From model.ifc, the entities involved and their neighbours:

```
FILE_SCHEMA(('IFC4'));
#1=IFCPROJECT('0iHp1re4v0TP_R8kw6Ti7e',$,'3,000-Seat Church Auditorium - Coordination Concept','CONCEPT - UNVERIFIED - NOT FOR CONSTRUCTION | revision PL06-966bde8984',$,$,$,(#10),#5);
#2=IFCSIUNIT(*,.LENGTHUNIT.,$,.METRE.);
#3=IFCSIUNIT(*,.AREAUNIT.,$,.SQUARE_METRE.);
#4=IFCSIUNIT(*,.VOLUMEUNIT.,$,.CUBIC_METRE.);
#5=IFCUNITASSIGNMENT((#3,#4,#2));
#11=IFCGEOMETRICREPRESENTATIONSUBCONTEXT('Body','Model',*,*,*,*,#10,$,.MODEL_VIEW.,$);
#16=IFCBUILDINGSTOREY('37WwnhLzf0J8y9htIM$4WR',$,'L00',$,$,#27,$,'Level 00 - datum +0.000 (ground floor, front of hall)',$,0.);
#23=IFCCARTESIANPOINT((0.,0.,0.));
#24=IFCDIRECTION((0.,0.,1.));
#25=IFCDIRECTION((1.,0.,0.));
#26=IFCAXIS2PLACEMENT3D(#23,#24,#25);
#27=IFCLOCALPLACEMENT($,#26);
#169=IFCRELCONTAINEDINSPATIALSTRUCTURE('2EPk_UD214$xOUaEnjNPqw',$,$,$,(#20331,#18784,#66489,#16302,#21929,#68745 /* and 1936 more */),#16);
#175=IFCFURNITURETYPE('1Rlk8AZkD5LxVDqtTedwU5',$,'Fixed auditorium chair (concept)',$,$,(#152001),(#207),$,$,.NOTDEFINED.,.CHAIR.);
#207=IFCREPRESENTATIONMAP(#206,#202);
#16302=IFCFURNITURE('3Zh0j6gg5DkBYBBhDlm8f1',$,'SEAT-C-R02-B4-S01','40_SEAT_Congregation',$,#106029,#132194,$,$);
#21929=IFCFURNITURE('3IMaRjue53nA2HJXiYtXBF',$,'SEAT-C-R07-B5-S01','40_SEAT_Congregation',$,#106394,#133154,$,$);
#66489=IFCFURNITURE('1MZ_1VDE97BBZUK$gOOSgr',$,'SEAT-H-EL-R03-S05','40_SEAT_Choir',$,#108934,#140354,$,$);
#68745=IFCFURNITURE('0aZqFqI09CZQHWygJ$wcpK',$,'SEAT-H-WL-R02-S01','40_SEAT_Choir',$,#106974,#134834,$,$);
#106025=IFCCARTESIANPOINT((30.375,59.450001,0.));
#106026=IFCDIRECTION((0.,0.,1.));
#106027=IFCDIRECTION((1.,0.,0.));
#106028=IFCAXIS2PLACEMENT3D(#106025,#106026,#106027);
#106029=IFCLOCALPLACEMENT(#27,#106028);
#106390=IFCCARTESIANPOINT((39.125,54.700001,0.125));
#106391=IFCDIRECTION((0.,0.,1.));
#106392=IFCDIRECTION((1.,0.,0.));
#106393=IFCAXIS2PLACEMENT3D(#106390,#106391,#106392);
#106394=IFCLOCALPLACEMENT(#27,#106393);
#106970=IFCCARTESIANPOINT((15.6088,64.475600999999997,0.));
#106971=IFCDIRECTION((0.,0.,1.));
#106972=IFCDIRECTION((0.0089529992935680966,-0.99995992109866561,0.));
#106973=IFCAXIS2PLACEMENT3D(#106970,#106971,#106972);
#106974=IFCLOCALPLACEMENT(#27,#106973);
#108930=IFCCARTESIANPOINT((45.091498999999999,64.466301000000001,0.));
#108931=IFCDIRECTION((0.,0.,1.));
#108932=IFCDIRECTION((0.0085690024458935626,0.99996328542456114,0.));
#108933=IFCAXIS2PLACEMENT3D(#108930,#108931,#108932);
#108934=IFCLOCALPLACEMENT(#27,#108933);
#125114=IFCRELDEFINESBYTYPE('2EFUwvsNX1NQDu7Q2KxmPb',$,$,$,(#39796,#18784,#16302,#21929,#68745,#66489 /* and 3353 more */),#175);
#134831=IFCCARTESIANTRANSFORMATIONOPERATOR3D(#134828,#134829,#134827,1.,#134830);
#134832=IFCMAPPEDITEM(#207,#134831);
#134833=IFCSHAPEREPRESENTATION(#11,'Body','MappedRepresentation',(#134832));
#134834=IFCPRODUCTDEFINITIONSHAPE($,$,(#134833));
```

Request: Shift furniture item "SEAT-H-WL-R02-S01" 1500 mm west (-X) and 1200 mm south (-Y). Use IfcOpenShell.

```python
import ifcopenshell
import ifcopenshell.api.geometry
import ifcopenshell.util.placement
import ifcopenshell.util.unit

model = ifcopenshell.open("model.ifc")
unit_scale = ifcopenshell.util.unit.calculate_unit_scale(model)

item = model.by_guid("0aZqFqI09CZQHWygJ$wcpK")
matrix = ifcopenshell.util.placement.get_local_placement(item.ObjectPlacement)
matrix[0, 3] -= 1.5 / unit_scale
matrix[1, 3] -= 1.2 / unit_scale
ifcopenshell.api.geometry.edit_object_placement(model, product=item, matrix=matrix, is_si=False)

print(ifcopenshell.util.placement.get_local_placement(item.ObjectPlacement).round(3) + 0.0)

model.write("model-out.ifc")
```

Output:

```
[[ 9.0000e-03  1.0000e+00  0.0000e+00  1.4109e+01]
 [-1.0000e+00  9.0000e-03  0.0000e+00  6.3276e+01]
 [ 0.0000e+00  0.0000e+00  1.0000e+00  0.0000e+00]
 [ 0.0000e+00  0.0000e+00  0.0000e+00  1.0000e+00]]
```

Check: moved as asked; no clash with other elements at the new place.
